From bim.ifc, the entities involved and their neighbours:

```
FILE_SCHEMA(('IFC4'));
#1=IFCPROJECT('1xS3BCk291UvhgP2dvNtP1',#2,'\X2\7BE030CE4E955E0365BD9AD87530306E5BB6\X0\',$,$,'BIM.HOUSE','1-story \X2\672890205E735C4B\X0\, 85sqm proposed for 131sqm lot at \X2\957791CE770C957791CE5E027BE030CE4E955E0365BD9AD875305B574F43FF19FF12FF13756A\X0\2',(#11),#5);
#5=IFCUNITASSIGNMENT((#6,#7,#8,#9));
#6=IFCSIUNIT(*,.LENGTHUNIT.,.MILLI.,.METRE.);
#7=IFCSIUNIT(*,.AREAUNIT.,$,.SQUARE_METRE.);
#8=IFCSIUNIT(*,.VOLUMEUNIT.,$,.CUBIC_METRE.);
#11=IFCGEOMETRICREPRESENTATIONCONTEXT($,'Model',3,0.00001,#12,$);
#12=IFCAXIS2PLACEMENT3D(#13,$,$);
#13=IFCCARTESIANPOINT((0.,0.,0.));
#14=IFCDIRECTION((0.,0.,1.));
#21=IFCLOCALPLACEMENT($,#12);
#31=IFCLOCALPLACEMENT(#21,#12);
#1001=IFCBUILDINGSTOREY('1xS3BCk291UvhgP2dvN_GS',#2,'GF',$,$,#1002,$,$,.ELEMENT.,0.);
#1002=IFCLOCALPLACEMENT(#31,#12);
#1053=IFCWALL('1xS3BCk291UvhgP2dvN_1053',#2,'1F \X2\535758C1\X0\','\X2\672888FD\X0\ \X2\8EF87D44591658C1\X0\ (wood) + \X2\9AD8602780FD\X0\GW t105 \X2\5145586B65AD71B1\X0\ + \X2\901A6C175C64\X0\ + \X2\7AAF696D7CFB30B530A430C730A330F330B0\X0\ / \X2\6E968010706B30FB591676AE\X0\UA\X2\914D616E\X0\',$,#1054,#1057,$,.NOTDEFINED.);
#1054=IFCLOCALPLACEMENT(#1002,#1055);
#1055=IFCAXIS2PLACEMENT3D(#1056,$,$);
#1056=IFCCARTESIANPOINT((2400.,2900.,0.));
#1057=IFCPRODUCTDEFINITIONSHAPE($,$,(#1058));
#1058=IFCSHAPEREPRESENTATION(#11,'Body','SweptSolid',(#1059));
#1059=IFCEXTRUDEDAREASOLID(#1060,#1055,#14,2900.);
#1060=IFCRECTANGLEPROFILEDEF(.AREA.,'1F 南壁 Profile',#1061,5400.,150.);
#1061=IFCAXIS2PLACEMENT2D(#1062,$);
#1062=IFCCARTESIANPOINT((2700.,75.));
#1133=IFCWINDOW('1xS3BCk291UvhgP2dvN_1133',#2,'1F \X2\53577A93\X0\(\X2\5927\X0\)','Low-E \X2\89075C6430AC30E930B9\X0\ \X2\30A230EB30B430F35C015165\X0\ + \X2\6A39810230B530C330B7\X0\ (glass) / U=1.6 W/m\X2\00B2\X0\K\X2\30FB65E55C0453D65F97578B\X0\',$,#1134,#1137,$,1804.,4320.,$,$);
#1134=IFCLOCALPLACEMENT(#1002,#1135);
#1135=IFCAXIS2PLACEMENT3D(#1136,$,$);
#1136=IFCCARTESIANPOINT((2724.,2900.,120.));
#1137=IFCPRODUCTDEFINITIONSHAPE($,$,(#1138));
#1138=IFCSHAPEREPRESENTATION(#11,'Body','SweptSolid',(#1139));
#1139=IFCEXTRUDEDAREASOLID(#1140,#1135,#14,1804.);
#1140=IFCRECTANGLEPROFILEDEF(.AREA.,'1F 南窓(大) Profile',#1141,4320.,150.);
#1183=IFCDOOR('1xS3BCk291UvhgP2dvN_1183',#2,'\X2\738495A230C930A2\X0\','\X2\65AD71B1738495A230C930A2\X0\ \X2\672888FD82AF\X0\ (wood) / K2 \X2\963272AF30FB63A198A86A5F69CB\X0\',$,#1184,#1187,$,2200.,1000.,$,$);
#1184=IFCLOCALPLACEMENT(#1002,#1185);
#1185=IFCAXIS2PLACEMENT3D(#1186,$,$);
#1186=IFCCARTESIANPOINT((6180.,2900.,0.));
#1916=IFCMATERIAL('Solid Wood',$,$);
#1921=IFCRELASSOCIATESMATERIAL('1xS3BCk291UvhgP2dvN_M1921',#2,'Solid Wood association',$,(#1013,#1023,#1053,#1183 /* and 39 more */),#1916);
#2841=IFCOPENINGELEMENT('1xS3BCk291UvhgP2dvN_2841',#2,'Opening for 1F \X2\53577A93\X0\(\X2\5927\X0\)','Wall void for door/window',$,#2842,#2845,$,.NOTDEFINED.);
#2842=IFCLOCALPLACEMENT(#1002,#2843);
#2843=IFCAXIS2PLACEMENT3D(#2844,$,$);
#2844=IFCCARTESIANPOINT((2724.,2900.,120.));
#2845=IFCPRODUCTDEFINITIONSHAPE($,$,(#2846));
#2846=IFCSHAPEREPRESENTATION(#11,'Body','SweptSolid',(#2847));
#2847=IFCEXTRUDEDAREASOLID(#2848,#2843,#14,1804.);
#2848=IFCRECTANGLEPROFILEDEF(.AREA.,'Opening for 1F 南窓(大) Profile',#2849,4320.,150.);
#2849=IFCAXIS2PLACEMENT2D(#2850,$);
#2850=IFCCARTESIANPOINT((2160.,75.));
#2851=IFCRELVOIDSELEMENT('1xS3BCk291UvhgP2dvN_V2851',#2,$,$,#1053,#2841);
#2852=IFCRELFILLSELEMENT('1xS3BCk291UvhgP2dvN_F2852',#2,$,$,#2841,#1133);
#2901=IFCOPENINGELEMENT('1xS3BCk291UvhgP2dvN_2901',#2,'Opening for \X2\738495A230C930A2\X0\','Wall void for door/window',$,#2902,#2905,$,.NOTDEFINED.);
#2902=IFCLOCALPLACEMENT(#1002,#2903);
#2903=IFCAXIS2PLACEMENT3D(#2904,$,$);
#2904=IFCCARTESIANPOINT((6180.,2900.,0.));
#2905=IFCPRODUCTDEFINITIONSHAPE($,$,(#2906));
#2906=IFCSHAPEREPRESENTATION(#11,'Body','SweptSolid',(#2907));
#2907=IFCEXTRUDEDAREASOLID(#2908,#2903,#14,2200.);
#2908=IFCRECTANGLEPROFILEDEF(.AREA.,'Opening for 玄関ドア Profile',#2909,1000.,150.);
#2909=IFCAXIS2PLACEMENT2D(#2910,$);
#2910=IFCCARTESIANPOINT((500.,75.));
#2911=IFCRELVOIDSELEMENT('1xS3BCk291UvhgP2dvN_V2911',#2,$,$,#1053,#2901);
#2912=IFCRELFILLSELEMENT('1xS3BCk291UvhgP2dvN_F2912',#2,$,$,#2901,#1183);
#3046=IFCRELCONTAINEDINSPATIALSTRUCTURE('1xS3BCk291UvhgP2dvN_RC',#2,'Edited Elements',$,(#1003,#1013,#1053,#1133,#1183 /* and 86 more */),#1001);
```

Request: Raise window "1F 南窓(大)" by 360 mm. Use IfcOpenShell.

```python
import numpy as np
import ifcopenshell
import ifcopenshell.api.geometry
import ifcopenshell.util.placement
import ifcopenshell.util.unit

model = ifcopenshell.open("bim.ifc")
unit_scale = ifcopenshell.util.unit.calculate_unit_scale(model)

window = model.by_guid("1xS3BCk291UvhgP2dvN_1133")
opening = window.FillsVoids[0].RelatingOpeningElement
dz = 360.0

shift = np.array([0.0, 0.0, dz])
# The window is not placed relative to its opening, so move both.
for product in (opening, window):
    matrix = ifcopenshell.util.placement.get_local_placement(product.ObjectPlacement)
    matrix[:3, 3] += shift
    ifcopenshell.api.geometry.edit_object_placement(model, product=product, matrix=matrix, is_si=False)

print(f"moved by {dz * unit_scale:+.3f} m")

model.write("bim_rev.ifc")
```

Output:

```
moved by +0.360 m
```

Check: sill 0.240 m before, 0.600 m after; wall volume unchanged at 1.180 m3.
